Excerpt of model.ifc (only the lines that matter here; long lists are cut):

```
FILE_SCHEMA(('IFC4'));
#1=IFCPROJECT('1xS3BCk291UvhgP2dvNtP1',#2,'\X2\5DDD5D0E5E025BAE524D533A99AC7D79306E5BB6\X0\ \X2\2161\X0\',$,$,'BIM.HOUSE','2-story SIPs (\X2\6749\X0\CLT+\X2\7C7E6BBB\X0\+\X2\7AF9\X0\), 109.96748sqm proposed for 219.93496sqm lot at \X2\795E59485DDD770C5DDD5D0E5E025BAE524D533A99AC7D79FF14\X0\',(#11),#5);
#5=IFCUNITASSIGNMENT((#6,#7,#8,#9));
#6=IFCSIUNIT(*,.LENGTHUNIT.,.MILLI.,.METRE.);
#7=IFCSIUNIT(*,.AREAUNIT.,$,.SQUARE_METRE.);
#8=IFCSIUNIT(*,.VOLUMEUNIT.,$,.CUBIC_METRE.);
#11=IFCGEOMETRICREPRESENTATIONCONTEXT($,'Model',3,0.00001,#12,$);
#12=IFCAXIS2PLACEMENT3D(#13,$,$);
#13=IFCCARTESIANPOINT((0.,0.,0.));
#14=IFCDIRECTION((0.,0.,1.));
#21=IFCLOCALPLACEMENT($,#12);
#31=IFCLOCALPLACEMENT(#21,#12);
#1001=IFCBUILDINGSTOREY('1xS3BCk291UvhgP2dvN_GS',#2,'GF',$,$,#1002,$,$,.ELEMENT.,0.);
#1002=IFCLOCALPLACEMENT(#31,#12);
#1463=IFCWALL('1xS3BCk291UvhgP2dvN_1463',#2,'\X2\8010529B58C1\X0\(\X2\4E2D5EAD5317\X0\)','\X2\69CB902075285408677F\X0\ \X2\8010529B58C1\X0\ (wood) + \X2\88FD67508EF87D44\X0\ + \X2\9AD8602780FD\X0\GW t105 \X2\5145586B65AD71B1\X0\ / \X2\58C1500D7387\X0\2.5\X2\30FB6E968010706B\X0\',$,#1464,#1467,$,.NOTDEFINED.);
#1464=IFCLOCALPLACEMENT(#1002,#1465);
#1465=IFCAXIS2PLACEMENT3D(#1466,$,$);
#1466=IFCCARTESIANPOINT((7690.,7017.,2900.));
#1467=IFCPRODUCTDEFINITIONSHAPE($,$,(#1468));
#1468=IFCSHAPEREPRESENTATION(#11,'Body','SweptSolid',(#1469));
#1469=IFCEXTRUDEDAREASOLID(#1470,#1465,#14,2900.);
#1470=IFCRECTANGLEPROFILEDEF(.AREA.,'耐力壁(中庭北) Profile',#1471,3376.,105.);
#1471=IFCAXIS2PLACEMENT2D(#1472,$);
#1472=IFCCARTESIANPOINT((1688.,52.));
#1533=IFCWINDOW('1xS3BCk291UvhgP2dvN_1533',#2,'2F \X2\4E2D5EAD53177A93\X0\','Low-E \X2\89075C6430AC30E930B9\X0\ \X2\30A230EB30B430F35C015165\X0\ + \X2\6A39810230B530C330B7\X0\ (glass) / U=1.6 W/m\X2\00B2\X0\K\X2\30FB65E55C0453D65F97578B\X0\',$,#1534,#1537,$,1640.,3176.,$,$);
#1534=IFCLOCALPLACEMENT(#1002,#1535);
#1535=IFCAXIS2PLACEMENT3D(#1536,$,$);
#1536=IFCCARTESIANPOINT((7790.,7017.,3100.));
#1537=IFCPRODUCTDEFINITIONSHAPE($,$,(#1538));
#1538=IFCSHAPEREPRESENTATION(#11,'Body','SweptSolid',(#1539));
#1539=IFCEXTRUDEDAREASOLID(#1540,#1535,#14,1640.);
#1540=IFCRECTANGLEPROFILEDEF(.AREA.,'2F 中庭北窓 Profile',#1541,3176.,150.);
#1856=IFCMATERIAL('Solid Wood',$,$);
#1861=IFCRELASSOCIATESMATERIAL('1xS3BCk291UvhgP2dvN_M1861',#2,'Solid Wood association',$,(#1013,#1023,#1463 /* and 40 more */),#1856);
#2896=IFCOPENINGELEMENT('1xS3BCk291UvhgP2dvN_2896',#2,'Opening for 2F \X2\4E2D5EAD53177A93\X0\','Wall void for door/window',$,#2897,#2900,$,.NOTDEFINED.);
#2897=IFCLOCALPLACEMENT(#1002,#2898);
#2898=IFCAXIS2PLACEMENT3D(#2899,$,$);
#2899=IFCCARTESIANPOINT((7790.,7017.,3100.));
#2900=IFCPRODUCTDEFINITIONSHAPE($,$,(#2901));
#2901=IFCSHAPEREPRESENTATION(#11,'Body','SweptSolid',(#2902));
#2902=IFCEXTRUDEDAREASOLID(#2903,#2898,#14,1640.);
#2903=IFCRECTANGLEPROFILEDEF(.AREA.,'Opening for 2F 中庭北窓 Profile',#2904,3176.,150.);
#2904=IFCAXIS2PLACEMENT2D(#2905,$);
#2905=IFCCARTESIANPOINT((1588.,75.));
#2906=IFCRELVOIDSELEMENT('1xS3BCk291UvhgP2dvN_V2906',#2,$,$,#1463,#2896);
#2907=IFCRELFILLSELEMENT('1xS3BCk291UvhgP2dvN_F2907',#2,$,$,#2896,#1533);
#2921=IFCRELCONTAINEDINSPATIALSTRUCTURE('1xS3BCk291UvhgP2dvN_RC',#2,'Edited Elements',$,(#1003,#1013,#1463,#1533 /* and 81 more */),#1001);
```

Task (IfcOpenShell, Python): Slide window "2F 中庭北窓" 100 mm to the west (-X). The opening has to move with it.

```python
import ifcopenshell
import ifcopenshell.api.geometry
import ifcopenshell.util.placement
import ifcopenshell.util.unit

model = ifcopenshell.open("model.ifc")
unit_scale = ifcopenshell.util.unit.calculate_unit_scale(model)

window = model.by_id(1533)
opening = window.FillsVoids[0].RelatingOpeningElement
wall = opening.VoidsElements[0].RelatingBuildingElement

wall_matrix = ifcopenshell.util.placement.get_local_placement(wall.ObjectPlacement)
shift = wall_matrix[:3, 0] * -0.1 / unit_scale
before = ifcopenshell.util.placement.get_local_placement(window.ObjectPlacement)[:3, 3].copy()

# The window is not placed relative to its opening, so move both.
for product in (opening, window):
    matrix = ifcopenshell.util.placement.get_local_placement(product.ObjectPlacement)
    matrix[:3, 3] += shift
    ifcopenshell.api.geometry.edit_object_placement(model, product=product, matrix=matrix, is_si=False)

after = ifcopenshell.util.placement.get_local_placement(window.ObjectPlacement)[:3, 3]
print("window moved by", (after - before).round(3) + 0.0)

model.write("model-out.ifc")
```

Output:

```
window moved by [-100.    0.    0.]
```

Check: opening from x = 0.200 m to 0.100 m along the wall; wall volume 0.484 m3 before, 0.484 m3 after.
